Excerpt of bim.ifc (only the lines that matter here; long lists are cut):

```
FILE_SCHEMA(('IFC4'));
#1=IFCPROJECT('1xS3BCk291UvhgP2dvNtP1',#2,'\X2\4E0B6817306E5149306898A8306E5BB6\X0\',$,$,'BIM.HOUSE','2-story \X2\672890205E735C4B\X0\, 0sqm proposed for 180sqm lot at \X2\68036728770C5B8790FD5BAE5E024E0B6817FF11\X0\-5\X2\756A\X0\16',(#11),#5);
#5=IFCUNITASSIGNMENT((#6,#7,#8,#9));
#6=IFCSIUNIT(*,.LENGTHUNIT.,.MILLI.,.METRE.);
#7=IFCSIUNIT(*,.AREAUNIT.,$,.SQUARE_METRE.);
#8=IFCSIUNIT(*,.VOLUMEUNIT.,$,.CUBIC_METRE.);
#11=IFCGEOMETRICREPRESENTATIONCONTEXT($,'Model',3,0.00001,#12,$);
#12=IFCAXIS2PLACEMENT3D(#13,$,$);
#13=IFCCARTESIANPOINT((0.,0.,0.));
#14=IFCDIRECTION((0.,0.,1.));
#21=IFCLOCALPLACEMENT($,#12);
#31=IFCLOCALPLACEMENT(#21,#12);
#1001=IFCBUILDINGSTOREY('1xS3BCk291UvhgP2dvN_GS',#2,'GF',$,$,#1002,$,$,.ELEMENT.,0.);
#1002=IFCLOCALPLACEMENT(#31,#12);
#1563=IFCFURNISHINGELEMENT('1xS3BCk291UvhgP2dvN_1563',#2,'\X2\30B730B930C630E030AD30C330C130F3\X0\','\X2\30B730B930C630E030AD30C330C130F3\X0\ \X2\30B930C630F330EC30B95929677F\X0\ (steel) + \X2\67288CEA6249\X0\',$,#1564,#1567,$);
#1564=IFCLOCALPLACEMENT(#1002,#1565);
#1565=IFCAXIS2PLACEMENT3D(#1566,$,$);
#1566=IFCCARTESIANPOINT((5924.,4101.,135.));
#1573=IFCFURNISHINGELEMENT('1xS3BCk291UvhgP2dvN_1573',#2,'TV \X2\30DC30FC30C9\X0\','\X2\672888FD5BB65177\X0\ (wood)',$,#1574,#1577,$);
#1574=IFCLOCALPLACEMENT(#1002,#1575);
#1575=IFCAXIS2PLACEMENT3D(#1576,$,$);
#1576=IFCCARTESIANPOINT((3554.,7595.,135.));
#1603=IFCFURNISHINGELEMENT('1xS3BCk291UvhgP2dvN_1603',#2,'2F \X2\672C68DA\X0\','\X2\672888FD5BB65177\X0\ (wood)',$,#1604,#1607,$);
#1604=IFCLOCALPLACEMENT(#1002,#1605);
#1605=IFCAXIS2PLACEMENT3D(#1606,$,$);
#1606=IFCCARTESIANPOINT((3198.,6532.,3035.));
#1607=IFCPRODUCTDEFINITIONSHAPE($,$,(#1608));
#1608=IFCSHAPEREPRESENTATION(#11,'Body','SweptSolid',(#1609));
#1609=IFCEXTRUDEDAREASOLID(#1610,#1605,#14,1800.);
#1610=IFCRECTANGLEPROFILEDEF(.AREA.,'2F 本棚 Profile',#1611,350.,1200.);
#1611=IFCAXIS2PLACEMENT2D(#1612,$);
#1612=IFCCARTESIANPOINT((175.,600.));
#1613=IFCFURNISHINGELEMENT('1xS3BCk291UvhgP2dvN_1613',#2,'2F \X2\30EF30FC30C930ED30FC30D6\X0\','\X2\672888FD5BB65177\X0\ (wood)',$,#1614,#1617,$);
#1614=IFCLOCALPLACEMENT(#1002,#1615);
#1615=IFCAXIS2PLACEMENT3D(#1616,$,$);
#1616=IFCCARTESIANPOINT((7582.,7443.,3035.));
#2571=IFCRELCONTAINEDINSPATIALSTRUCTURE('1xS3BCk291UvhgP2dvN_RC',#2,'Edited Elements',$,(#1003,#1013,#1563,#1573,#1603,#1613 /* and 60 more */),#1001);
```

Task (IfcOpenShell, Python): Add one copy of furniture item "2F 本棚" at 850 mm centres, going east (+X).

```python
import numpy as np
import ifcopenshell
import ifcopenshell.api.geometry
import ifcopenshell.api.root
import ifcopenshell.util.element
import ifcopenshell.util.placement
import ifcopenshell.util.unit

model = ifcopenshell.open("bim.ifc")
unit_scale = ifcopenshell.util.unit.calculate_unit_scale(model)


def reuse_history(source, copy):
    """copy_class also copies each property set's owner history, people and application; keep the originals."""
    for rel in copy.IsDefinedBy:
        if rel.is_a("IfcRelDefinesByProperties") and (history := rel.RelatingPropertyDefinition.OwnerHistory):
            rel.RelatingPropertyDefinition.OwnerHistory = source.OwnerHistory
            ifcopenshell.util.element.remove_deep2(model, history)


source = model.by_id(1603)
base = ifcopenshell.util.placement.get_local_placement(source.ObjectPlacement)
step = np.array([1.0, 0.0, 0.0]) * 0.85 / unit_scale

for i in range(1, 2):
    copy = ifcopenshell.api.root.copy_class(model, product=source)
    copy.Representation = ifcopenshell.util.element.copy_deep(
        model, source.Representation, exclude=["IfcGeometricRepresentationContext", "IfcRepresentationMap"]
    )
    reuse_history(source, copy)
    matrix = base.copy()
    matrix[:3, 3] += i * step
    print("added at", matrix[:3, 3].round(3) + 0.0)
    ifcopenshell.api.geometry.edit_object_placement(model, product=copy, matrix=matrix, is_si=False)

model.write("bim_edited.ifc")
```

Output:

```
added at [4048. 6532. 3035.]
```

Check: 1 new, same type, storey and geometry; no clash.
